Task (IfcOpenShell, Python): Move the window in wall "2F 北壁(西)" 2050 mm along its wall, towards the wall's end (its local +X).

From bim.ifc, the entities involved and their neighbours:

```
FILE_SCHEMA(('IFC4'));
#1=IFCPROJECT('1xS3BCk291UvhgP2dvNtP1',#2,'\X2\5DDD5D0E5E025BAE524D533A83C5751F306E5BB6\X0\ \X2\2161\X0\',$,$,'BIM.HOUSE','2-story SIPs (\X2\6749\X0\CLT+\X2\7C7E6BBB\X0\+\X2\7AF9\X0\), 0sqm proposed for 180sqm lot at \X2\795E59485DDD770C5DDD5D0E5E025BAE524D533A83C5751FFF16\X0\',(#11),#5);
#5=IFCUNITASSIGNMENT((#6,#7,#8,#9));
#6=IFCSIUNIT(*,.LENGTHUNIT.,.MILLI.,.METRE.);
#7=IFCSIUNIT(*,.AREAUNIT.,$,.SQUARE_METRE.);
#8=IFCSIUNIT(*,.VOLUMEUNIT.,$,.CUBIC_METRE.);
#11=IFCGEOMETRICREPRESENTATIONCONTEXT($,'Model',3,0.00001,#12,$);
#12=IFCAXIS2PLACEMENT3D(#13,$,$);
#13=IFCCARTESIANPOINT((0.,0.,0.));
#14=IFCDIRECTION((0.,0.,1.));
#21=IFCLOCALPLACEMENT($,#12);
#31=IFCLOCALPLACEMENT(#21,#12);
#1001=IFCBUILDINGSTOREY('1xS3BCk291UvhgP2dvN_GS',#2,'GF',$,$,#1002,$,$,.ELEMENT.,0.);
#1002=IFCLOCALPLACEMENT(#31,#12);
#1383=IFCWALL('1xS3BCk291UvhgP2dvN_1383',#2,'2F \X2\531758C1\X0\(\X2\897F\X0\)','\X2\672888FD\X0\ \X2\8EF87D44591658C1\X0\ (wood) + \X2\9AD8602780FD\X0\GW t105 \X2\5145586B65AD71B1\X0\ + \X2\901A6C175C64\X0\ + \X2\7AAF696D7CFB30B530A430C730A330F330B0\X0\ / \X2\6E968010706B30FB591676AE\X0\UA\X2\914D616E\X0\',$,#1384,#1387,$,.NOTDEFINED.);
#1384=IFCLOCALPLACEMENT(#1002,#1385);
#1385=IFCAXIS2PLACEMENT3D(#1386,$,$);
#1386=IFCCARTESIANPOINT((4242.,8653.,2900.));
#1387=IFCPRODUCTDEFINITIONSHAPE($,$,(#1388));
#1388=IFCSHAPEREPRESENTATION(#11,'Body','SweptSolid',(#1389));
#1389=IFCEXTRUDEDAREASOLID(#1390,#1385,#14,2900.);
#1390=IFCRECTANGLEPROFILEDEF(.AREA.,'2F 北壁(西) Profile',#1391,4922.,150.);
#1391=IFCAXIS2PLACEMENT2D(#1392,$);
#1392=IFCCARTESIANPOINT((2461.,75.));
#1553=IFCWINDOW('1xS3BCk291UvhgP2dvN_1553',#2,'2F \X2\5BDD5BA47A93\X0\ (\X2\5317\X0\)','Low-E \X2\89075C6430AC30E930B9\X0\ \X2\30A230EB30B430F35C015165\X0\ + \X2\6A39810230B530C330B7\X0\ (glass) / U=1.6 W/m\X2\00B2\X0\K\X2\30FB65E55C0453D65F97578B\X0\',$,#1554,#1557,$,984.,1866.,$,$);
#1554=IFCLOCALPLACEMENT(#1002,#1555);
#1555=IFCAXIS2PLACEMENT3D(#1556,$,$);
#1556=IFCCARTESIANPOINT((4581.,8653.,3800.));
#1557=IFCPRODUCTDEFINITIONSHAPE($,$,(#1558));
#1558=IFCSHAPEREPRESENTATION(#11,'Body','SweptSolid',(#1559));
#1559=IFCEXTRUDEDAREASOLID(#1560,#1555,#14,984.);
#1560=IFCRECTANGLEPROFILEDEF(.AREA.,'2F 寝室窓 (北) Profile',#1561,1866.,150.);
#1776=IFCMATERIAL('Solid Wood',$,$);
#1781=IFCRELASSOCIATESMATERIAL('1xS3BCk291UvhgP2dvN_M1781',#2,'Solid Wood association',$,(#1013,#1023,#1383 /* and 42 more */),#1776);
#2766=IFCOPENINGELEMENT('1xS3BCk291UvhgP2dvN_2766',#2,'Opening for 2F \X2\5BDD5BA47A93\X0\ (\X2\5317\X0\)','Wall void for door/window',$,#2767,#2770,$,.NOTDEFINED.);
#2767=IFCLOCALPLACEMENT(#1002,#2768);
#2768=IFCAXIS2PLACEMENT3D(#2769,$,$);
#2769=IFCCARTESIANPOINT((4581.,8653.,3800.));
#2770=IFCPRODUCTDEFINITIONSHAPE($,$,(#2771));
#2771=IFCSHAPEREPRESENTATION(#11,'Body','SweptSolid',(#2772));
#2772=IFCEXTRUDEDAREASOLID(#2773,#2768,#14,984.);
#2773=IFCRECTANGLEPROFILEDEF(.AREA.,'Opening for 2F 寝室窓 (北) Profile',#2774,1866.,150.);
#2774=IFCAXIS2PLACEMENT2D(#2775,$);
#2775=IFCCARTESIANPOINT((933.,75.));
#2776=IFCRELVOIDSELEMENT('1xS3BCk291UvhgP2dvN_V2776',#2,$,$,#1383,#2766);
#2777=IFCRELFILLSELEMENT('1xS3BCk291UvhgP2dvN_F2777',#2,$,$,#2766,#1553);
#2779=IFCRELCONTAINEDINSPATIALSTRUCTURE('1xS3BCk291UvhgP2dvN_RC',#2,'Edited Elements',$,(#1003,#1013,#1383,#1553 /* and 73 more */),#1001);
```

```python
import ifcopenshell
import ifcopenshell.api.geometry
import ifcopenshell.util.placement
import ifcopenshell.util.unit

model = ifcopenshell.open("bim.ifc")
unit_scale = ifcopenshell.util.unit.calculate_unit_scale(model)

window = model.by_guid("1xS3BCk291UvhgP2dvN_1553")
opening = window.FillsVoids[0].RelatingOpeningElement
wall = opening.VoidsElements[0].RelatingBuildingElement

wall_matrix = ifcopenshell.util.placement.get_local_placement(wall.ObjectPlacement)
shift = wall_matrix[:3, 0] * 2.05 / unit_scale
before = ifcopenshell.util.placement.get_local_placement(window.ObjectPlacement)[:3, 3].copy()

# The window is not placed relative to its opening, so move both.
for product in (opening, window):
    matrix = ifcopenshell.util.placement.get_local_placement(product.ObjectPlacement)
    matrix[:3, 3] += shift
    ifcopenshell.api.geometry.edit_object_placement(model, product=product, matrix=matrix, is_si=False)

after = ifcopenshell.util.placement.get_local_placement(window.ObjectPlacement)[:3, 3]
print("window moved by", (after - before).round(3) + 0.0)

model.write("bim_rev.ifc")
```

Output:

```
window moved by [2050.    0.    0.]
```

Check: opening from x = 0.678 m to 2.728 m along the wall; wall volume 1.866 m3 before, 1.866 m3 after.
